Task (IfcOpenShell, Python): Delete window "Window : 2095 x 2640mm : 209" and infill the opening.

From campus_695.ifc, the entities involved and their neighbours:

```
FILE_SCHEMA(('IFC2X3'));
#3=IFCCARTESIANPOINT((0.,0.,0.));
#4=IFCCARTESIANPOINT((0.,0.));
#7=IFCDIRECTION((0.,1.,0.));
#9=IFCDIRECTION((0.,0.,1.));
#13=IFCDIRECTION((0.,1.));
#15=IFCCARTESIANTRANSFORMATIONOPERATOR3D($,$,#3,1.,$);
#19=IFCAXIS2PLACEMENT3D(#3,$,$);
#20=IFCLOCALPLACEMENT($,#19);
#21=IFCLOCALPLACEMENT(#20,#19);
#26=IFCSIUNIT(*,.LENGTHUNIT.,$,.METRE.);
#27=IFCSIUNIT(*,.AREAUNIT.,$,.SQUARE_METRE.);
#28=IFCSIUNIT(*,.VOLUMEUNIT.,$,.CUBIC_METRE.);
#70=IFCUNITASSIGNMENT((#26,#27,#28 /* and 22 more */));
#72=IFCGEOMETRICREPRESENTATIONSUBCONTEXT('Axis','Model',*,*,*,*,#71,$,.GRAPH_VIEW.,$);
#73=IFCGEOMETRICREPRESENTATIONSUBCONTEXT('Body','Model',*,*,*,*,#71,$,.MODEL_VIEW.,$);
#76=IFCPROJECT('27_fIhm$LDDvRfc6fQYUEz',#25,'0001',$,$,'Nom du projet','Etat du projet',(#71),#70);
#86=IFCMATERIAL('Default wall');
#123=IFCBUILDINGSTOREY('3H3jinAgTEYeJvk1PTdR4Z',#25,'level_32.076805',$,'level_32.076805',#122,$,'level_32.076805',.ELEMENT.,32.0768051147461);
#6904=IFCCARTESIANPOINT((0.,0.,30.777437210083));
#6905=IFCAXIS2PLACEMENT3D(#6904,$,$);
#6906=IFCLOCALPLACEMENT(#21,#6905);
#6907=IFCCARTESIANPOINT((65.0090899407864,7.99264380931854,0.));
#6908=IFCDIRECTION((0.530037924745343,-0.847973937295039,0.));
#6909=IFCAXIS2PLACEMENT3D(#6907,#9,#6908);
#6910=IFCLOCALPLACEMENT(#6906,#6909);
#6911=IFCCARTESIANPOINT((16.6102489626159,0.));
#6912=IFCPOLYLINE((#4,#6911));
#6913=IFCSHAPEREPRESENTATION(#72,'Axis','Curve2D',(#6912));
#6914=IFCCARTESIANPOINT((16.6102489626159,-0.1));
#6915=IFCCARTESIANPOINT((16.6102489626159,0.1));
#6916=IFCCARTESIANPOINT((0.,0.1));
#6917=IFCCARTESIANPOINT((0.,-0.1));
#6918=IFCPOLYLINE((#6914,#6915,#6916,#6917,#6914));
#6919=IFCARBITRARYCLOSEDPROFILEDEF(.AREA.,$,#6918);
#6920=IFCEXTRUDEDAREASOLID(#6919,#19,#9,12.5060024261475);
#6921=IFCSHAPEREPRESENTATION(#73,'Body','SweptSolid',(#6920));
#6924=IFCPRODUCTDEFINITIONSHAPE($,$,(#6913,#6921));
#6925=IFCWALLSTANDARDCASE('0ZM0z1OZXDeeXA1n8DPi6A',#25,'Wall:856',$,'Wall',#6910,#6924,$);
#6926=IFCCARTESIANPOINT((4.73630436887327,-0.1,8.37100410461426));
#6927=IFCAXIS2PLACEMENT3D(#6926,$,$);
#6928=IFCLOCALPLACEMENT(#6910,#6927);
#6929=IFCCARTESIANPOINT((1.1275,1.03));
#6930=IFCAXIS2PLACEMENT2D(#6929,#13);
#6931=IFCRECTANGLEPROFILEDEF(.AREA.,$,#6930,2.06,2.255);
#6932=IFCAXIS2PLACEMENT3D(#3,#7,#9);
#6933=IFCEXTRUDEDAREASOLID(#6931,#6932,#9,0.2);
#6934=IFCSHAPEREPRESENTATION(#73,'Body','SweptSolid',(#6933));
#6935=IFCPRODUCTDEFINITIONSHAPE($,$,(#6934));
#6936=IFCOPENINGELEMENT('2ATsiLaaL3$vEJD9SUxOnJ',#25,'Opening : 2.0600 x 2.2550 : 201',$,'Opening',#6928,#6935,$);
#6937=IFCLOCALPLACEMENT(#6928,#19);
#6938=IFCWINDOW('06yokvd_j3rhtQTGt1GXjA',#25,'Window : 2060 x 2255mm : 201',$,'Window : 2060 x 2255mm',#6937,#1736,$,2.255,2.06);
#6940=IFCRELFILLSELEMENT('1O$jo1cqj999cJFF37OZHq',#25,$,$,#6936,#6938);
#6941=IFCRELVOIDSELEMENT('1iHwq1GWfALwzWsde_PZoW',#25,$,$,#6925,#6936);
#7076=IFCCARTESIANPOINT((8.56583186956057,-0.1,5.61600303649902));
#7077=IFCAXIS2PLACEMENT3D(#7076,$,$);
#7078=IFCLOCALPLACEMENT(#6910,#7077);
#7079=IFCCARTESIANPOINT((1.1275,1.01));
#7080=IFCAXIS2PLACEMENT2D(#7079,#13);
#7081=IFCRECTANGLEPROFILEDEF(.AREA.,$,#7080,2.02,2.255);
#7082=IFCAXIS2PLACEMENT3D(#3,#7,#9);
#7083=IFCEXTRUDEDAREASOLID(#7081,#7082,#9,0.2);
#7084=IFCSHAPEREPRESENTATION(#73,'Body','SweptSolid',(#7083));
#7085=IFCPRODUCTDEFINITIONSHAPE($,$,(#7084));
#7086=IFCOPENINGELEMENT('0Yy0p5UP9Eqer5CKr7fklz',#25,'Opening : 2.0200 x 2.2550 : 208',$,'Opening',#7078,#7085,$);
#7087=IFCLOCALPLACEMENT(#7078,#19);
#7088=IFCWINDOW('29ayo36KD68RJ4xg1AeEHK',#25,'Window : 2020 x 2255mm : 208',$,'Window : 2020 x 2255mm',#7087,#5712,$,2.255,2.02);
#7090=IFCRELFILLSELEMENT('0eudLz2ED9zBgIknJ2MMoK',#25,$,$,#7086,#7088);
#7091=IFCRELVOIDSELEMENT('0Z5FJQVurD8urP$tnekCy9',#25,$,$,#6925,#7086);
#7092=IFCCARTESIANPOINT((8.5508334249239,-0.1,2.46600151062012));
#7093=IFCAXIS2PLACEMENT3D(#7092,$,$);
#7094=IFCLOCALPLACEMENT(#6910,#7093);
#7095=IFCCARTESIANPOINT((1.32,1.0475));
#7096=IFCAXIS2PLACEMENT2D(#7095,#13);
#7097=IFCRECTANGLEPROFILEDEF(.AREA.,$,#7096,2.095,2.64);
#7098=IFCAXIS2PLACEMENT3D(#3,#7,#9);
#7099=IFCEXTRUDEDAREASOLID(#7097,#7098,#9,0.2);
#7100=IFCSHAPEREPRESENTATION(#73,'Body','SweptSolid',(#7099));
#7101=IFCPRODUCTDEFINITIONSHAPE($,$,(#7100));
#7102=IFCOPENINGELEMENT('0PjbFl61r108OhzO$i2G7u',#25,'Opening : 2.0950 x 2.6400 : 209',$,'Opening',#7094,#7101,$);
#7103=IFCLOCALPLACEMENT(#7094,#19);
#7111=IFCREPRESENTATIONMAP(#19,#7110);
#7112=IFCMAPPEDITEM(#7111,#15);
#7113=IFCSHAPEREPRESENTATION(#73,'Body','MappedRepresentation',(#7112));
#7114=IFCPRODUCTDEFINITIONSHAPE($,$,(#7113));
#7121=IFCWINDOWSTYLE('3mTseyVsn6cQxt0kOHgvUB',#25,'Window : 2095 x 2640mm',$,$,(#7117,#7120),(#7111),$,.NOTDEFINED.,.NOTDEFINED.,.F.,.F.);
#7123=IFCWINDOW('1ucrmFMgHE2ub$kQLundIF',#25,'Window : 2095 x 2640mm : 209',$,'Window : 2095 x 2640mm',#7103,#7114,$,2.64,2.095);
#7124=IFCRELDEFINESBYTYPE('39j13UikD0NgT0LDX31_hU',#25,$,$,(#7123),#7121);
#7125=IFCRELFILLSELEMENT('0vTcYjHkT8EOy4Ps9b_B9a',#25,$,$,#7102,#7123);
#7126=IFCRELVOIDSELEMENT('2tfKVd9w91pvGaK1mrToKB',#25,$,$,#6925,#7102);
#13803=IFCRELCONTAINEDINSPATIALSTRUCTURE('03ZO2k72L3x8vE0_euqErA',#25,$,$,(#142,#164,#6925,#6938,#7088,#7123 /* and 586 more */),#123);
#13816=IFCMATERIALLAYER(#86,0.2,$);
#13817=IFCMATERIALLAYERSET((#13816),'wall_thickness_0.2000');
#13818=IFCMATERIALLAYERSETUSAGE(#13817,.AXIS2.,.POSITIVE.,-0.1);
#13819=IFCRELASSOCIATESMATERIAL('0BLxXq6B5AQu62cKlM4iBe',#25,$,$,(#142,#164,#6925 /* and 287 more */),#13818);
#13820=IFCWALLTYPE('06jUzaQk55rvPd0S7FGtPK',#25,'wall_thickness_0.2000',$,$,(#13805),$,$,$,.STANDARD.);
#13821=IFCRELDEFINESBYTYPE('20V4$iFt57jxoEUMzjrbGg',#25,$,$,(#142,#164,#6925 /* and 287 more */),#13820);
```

```python
import ifcopenshell
import ifcopenshell.api.feature
import ifcopenshell.api.root
import ifcopenshell.geom
import ifcopenshell.util.shape

model = ifcopenshell.open("campus_695.ifc")
settings = ifcopenshell.geom.settings()


def volume(element):
    """Net volume in cubic metres, openings subtracted."""
    shape = ifcopenshell.geom.create_shape(settings, element)
    return ifcopenshell.util.shape.get_volume(shape.geometry)


window = model.by_guid("1ucrmFMgHE2ub$kQLundIF")
opening = window.FillsVoids[0].RelatingOpeningElement
wall = opening.VoidsElements[0].RelatingBuildingElement
before = volume(wall)

ifcopenshell.api.root.remove_product(model, product=window)
ifcopenshell.api.feature.remove_feature(model, feature=opening)

after = volume(wall)

print(f"wall volume {before:.3f} -> {after:.3f} m3")

model.write("campus_695_edited.ifc")
```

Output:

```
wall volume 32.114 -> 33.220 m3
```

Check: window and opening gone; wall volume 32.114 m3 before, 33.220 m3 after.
